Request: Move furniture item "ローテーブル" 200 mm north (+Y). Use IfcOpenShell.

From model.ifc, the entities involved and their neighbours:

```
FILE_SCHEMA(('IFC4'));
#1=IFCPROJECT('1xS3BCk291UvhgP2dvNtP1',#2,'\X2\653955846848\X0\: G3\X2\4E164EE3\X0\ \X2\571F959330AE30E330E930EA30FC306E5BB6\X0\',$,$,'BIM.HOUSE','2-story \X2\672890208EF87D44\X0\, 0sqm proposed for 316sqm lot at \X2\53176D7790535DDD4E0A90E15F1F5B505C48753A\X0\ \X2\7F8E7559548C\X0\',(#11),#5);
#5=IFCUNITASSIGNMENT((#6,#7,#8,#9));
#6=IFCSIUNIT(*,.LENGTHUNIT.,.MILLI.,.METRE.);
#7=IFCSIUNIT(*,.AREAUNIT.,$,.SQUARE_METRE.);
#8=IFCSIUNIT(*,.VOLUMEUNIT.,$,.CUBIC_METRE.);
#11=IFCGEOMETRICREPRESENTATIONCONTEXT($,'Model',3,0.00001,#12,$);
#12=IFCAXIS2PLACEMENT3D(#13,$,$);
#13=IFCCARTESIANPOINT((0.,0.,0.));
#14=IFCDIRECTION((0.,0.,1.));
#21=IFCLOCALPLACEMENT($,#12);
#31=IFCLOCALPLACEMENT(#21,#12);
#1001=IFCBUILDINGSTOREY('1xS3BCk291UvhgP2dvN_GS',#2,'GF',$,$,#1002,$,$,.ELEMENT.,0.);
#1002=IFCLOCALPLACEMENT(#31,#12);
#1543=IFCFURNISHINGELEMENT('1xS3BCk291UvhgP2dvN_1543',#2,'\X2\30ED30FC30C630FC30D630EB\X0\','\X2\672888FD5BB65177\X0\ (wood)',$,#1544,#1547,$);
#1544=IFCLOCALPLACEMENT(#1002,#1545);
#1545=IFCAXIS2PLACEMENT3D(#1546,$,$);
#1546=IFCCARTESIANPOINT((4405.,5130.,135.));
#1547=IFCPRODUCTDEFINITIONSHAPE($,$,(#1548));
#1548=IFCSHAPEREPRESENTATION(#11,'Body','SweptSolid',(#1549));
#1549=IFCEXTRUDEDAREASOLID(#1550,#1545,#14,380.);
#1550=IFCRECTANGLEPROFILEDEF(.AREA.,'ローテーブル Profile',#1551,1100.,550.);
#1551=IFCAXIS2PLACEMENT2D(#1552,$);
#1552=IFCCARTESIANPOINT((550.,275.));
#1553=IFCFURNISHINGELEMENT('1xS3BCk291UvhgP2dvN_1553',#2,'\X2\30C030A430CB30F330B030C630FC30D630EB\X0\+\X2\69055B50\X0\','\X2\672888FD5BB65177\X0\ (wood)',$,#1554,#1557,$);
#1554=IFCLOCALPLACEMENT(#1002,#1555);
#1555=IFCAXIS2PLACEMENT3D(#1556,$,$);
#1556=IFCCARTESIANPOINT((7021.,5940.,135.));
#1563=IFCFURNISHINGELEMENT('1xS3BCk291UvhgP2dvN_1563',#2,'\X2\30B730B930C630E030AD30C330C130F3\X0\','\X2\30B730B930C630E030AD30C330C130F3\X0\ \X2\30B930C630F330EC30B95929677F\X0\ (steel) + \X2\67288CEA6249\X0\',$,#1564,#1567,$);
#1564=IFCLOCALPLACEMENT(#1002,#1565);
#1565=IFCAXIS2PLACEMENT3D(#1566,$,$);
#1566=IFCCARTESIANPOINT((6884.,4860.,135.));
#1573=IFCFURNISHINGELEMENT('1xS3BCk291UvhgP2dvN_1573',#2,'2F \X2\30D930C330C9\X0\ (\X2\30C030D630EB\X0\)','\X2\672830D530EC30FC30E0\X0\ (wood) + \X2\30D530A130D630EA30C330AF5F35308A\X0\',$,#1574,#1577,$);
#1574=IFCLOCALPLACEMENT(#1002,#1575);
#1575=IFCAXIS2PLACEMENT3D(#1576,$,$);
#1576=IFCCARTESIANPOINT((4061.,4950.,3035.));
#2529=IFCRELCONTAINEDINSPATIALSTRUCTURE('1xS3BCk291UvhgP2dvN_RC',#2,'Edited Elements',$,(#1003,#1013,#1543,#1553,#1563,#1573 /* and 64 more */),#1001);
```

```python
import ifcopenshell
import ifcopenshell.api.geometry
import ifcopenshell.util.placement
import ifcopenshell.util.unit

model = ifcopenshell.open("model.ifc")
unit_scale = ifcopenshell.util.unit.calculate_unit_scale(model)

item = model.by_guid("1xS3BCk291UvhgP2dvN_1543")
matrix = ifcopenshell.util.placement.get_local_placement(item.ObjectPlacement)
matrix[1, 3] += 0.2 / unit_scale
ifcopenshell.api.geometry.edit_object_placement(model, product=item, matrix=matrix, is_si=False)

print(ifcopenshell.util.placement.get_local_placement(item.ObjectPlacement).round(3) + 0.0)

model.write("model_v2.ifc")
```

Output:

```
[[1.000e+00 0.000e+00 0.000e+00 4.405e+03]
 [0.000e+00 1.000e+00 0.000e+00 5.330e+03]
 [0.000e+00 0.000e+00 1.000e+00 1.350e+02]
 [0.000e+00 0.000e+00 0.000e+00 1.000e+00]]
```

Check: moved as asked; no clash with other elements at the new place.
